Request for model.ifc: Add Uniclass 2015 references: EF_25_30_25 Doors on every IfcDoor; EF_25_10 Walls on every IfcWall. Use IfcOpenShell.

First a look at what the model holds.

```python
import ifcopenshell

model = ifcopenshell.open("model.ifc")
print(model.schema)
print("classifications:", [c.Name for c in model.by_type("IfcClassification")])
for ifc_class in ("IfcDoor", "IfcRoof", "IfcStair", "IfcWall", "IfcWindow"):
    print(ifc_class, len(model.by_type(ifc_class)))
```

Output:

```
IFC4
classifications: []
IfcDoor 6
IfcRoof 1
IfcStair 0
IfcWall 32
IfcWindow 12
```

```python
import ifcopenshell
import ifcopenshell.api.classification

model = ifcopenshell.open("model.ifc")

system = ifcopenshell.api.classification.add_classification(model, classification="Uniclass 2015")

codes = {
    "IfcDoor": ("EF_25_30_25", "Doors"),
    "IfcWall": ("EF_25_10", "Walls"),
}
for ifc_class, (code, name) in codes.items():
    products = model.by_type(ifc_class)
    ifcopenshell.api.classification.add_reference(
        model, products=products, classification=system, identification=code, name=name
    )
    print(code, len(products))

model.write("model-out.ifc")
```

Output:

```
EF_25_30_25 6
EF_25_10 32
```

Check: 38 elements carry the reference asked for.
